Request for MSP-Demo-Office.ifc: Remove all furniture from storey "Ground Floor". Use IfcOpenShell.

First a look at what the model holds.

```python
import ifcopenshell
import ifcopenshell.util.element

model = ifcopenshell.open("MSP-Demo-Office.ifc")
print(model.schema)
storey = next(s for s in model.by_type("IfcBuildingStorey") if s.Name == "Ground Floor")
furniture = [e for e in ifcopenshell.util.element.get_decomposition(storey) if e.is_a("IfcFurnishingElement")]
seen = {}
for e in furniture:
    element_type = ifcopenshell.util.element.get_type(e)
    name = element_type.Name if element_type not in (None, e) else None
    seen[name] = seen.get(name, 0) + 1
for name, count in sorted(seen.items(), key=str):
    print(count, "x", name)
```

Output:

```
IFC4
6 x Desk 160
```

```python
import ifcopenshell
import ifcopenshell.api.root
import ifcopenshell.util.element

model = ifcopenshell.open("MSP-Demo-Office.ifc")

storey = next(s for s in model.by_type("IfcBuildingStorey") if s.Name == "Ground Floor")
furniture = [e for e in ifcopenshell.util.element.get_decomposition(storey) if e.is_a("IfcFurnishingElement")]

for e in furniture:
    ifcopenshell.api.root.remove_product(model, product=e)
print(len(furniture), "removed")

model.write("MSP-Demo-Office-out.ifc")
```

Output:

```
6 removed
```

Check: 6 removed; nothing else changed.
